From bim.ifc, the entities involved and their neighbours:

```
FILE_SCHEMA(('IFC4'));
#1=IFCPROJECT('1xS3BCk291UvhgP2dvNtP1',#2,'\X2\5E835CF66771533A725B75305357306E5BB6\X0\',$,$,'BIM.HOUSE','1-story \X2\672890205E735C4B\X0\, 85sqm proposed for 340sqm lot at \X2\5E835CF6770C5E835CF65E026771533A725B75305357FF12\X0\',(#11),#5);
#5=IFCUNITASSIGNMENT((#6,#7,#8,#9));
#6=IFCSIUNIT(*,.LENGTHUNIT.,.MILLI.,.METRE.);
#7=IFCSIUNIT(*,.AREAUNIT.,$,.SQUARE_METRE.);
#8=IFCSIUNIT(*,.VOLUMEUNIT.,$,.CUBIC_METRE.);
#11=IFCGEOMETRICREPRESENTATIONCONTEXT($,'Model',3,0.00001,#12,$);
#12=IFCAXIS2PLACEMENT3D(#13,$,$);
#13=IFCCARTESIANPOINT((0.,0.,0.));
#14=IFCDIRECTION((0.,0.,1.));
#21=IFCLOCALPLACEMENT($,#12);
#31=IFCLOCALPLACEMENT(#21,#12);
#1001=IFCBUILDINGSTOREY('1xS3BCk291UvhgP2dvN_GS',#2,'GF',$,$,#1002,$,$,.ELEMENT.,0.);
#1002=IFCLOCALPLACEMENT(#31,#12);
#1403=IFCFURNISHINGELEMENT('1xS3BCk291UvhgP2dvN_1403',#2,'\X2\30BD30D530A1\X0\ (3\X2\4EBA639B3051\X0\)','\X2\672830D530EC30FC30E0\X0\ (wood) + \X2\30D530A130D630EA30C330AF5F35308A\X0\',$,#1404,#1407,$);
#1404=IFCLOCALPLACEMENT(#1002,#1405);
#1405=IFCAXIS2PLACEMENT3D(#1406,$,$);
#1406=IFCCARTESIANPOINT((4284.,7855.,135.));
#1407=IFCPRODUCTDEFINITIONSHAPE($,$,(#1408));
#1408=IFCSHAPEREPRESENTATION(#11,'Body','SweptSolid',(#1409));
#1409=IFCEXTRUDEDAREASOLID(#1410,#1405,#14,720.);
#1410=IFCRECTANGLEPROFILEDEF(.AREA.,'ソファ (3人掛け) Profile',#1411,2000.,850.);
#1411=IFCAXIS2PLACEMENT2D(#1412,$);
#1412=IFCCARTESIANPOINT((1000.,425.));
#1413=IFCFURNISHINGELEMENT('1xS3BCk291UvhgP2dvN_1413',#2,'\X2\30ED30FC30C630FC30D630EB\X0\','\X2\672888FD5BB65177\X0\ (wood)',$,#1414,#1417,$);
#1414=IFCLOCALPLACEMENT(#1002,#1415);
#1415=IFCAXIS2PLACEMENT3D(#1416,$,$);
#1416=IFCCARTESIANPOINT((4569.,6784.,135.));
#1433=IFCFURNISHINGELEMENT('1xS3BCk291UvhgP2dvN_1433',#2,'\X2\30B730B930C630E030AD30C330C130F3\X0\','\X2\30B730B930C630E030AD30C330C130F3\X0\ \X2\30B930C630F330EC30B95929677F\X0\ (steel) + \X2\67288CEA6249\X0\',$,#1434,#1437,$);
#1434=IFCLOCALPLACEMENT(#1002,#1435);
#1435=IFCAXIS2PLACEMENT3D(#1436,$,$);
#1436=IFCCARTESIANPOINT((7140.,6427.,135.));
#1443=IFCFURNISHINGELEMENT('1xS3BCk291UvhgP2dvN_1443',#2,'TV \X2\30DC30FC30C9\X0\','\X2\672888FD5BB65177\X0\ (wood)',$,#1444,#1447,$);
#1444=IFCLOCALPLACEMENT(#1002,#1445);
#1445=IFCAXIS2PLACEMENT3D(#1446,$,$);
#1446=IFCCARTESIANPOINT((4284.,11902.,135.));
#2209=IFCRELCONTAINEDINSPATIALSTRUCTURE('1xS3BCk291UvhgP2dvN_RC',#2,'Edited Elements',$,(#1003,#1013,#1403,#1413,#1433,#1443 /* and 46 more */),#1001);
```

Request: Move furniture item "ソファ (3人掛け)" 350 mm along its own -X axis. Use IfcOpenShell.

```python
import ifcopenshell
import ifcopenshell.api.geometry
import ifcopenshell.util.placement

model = ifcopenshell.open("bim.ifc")

item = model.by_id(1403)
matrix = ifcopenshell.util.placement.get_local_placement(item.ObjectPlacement)
matrix[:3, 3] -= matrix[:3, 0] * 350.0
ifcopenshell.api.geometry.edit_object_placement(model, product=item, matrix=matrix, is_si=False)

print(ifcopenshell.util.placement.get_local_placement(item.ObjectPlacement).round(3) + 0.0)

model.write("bim-out.ifc")
```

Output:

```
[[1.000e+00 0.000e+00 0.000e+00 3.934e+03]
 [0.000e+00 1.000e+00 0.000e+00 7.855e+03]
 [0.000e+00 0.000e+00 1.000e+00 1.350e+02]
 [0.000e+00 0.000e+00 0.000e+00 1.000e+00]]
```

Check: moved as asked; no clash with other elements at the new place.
